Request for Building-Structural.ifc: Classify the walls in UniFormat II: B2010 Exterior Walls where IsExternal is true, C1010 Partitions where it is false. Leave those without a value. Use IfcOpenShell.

First a look at what the model holds.

```python
import ifcopenshell
import ifcopenshell.util.element

model = ifcopenshell.open("Building-Structural.ifc")
print(model.schema)
print("classifications:", [c.Name for c in model.by_type("IfcClassification")])
values = [ifcopenshell.util.element.get_pset(e, "Pset_WallCommon", "IsExternal") for e in model.by_type("IfcWall")]
for value in (True, False, None):
    print("IsExternal", value, values.count(value))
```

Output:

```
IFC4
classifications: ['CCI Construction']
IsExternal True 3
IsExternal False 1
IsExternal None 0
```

```python
import ifcopenshell
import ifcopenshell.api.classification
import ifcopenshell.util.element

model = ifcopenshell.open("Building-Structural.ifc")

system = ifcopenshell.api.classification.add_classification(model, classification="UniFormat II")

walls = model.by_type("IfcWall")
external = {e: ifcopenshell.util.element.get_pset(e, "Pset_WallCommon", "IsExternal") for e in walls}
for flag, code, name in ((True, "B2010", "Exterior Walls"), (False, "C1010", "Partitions")):
    products = [e for e in walls if external[e] is flag]
    ifcopenshell.api.classification.add_reference(
        model, products=products, classification=system, identification=code, name=name
    )
    print(code, len(products))

model.write("Building-Structural_updated.ifc")
```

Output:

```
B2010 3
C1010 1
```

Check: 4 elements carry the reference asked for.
